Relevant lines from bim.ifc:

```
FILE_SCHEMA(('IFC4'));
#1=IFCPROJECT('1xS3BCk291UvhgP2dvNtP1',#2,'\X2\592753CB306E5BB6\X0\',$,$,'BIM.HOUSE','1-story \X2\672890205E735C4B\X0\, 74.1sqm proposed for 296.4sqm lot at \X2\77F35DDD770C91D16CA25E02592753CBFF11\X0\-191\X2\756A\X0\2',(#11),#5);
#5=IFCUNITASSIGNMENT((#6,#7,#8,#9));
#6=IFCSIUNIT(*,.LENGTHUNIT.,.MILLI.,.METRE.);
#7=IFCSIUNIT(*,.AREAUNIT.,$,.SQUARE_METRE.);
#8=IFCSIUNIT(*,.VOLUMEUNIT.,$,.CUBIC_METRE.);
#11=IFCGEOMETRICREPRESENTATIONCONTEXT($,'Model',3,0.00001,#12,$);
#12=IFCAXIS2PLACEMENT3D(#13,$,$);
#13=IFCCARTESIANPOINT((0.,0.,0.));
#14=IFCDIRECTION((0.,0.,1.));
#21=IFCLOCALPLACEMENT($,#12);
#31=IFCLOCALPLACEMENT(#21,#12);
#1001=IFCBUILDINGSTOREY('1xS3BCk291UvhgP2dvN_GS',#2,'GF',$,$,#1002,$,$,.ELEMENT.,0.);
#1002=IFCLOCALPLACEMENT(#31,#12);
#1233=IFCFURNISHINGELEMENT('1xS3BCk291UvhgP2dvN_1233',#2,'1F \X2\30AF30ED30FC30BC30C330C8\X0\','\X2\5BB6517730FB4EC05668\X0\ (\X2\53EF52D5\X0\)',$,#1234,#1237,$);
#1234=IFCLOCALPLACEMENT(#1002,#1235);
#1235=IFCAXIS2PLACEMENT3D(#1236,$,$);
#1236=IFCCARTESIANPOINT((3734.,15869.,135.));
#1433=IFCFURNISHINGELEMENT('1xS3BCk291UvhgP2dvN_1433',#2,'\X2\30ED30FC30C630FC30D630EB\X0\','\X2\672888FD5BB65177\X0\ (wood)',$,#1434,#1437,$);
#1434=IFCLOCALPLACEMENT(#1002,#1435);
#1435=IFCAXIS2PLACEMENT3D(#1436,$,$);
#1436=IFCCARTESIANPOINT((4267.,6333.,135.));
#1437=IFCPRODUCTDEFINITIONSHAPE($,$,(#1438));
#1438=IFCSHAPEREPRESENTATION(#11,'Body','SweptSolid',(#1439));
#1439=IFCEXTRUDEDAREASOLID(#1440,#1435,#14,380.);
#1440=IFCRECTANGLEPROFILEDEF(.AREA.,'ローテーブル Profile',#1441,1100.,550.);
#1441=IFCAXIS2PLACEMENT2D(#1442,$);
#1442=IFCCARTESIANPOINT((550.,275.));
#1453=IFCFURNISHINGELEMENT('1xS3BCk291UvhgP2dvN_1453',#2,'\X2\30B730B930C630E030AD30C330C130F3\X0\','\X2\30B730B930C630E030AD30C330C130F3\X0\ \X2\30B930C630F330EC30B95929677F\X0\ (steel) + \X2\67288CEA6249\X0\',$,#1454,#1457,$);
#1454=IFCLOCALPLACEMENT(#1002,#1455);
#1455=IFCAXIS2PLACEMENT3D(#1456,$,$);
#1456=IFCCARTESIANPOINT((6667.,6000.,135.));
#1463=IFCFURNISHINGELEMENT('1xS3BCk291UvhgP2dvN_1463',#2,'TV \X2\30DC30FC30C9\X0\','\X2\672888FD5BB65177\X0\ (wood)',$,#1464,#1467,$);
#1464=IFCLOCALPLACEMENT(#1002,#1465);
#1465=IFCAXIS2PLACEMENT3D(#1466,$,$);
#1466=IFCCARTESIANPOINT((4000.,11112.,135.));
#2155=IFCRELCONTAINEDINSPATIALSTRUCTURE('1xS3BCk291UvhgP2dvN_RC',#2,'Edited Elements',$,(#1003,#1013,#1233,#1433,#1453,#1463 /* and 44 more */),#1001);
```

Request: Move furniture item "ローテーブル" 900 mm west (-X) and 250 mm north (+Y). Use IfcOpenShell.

```python
import ifcopenshell
import ifcopenshell.api.geometry
import ifcopenshell.util.placement

model = ifcopenshell.open("bim.ifc")

item = model.by_guid("1xS3BCk291UvhgP2dvN_1433")
matrix = ifcopenshell.util.placement.get_local_placement(item.ObjectPlacement)
matrix[0, 3] -= 900.0
matrix[1, 3] += 250.0
ifcopenshell.api.geometry.edit_object_placement(model, product=item, matrix=matrix, is_si=False)

print(ifcopenshell.util.placement.get_local_placement(item.ObjectPlacement).round(3) + 0.0)

model.write("bim_edited.ifc")
```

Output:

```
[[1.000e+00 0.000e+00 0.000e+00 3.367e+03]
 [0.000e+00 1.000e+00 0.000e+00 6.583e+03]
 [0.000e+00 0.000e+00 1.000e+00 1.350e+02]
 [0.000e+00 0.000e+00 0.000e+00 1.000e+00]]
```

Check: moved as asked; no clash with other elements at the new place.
